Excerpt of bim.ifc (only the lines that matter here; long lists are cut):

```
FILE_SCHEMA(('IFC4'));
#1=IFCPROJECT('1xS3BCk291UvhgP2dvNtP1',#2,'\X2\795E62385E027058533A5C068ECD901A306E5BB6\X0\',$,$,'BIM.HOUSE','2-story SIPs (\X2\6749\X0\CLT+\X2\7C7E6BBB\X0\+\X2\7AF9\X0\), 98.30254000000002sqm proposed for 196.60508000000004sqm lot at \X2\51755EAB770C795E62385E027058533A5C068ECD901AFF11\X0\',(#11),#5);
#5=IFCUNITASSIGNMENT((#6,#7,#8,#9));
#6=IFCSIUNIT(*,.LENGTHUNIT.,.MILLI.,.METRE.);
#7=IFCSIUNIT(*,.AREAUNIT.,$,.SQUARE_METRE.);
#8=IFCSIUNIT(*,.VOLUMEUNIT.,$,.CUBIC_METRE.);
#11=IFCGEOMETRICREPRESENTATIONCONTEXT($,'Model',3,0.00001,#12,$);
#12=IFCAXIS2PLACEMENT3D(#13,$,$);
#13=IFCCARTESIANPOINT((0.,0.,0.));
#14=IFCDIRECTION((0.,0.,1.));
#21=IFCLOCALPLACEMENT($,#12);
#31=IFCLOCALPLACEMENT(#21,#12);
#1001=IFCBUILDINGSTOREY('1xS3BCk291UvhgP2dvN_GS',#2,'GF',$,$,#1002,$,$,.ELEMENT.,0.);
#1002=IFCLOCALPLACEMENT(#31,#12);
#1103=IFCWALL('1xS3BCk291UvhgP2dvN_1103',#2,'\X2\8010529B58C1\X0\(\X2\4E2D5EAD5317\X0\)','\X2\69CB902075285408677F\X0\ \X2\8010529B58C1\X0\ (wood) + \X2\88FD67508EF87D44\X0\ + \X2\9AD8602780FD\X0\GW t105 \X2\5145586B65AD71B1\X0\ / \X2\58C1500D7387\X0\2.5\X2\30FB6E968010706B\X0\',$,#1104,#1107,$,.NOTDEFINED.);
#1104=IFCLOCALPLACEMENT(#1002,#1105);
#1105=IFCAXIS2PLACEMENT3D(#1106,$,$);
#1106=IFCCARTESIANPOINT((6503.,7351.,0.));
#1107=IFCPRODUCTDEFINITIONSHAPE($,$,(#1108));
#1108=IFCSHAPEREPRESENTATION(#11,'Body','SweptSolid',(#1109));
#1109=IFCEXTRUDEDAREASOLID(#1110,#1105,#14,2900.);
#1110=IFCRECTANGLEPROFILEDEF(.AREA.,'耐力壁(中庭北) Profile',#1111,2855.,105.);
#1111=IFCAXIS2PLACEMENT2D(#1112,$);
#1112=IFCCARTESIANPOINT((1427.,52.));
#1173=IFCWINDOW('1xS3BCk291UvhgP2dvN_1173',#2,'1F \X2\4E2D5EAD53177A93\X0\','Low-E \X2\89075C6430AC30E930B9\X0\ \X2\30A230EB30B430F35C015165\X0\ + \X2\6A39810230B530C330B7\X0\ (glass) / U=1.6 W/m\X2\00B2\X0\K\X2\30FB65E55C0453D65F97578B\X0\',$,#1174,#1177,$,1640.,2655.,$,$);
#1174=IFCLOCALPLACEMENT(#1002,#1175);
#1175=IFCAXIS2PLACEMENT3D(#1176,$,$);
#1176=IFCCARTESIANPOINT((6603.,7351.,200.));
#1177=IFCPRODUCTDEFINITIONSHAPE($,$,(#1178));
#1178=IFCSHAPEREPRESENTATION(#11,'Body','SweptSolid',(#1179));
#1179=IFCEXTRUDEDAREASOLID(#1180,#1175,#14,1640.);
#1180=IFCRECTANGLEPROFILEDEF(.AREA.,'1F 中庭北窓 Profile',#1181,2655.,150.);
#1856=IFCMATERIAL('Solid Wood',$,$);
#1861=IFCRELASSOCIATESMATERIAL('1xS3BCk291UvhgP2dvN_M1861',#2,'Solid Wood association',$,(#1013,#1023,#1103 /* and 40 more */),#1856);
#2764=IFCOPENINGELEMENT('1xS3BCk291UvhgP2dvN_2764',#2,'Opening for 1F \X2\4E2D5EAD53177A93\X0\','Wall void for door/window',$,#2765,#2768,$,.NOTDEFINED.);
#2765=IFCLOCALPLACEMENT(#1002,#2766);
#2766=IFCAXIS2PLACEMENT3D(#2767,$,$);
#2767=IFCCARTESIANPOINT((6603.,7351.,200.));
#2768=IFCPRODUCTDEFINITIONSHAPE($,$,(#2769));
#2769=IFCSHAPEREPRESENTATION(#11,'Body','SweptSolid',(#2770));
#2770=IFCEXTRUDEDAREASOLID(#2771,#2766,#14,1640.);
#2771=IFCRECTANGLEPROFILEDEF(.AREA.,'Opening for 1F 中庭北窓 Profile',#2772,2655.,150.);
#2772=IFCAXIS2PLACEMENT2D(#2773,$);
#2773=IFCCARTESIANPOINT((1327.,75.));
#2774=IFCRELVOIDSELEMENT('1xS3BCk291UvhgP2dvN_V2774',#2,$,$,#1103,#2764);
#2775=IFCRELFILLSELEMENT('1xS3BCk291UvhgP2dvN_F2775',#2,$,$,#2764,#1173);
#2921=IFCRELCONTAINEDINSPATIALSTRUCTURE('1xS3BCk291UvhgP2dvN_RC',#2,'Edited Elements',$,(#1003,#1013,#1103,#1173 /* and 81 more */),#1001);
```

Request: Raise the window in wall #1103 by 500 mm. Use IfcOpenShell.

```python
import numpy as np
import ifcopenshell
import ifcopenshell.api.geometry
import ifcopenshell.util.placement
import ifcopenshell.util.unit

model = ifcopenshell.open("bim.ifc")
unit_scale = ifcopenshell.util.unit.calculate_unit_scale(model)

window = model.by_guid("1xS3BCk291UvhgP2dvN_1173")
opening = window.FillsVoids[0].RelatingOpeningElement
dz = 0.5 / unit_scale

shift = np.array([0.0, 0.0, dz])
# The window is not placed relative to its opening, so move both.
for product in (opening, window):
    matrix = ifcopenshell.util.placement.get_local_placement(product.ObjectPlacement)
    matrix[:3, 3] += shift
    ifcopenshell.api.geometry.edit_object_placement(model, product=product, matrix=matrix, is_si=False)

print(f"moved by {dz * unit_scale:+.3f} m")

model.write("bim_edited.ifc")
```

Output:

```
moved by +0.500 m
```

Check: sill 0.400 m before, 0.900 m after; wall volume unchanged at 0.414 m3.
